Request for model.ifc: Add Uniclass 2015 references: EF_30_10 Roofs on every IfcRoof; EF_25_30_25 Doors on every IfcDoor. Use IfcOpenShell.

First a look at what the model holds.

```python
import ifcopenshell

model = ifcopenshell.open("model.ifc")
print(model.schema)
print("classifications:", [c.Name for c in model.by_type("IfcClassification")])
for ifc_class in ("IfcDoor", "IfcRoof", "IfcStair", "IfcWall", "IfcWindow"):
    print(ifc_class, len(model.by_type(ifc_class)))
```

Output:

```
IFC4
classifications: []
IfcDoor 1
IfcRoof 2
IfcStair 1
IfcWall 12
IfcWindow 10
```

```python
import ifcopenshell
import ifcopenshell.api.classification

model = ifcopenshell.open("model.ifc")

system = ifcopenshell.api.classification.add_classification(model, classification="Uniclass 2015")

codes = {
    "IfcRoof": ("EF_30_10", "Roofs"),
    "IfcDoor": ("EF_25_30_25", "Doors"),
}
for ifc_class, (code, name) in codes.items():
    products = model.by_type(ifc_class)
    ifcopenshell.api.classification.add_reference(
        model, products=products, classification=system, identification=code, name=name
    )
    print(code, len(products))

model.write("model_v2.ifc")
```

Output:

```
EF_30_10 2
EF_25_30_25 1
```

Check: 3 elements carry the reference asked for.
